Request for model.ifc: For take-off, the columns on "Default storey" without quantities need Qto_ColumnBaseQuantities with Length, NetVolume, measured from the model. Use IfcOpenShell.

First a look at what the model holds.

```python
import ifcopenshell
import ifcopenshell.util.element
import ifcopenshell.util.unit

model = ifcopenshell.open("model.ifc")
print(model.schema)
for unit_type in ("LENGTHUNIT", "AREAUNIT", "VOLUMEUNIT"):
    print(unit_type, ifcopenshell.util.unit.calculate_unit_scale(model, unit_type))
storey = next(s for s in model.by_type("IfcBuildingStorey") if s.Name == "Default storey")
columns = [e for e in ifcopenshell.util.element.get_decomposition(storey) if e.is_a("IfcColumn")]
for e in sorted(columns, key=lambda e: e.id()):
    print(e.id(), e.is_a(), e.Name, list(ifcopenshell.util.element.get_psets(e, qtos_only=True)), sep=" | ")
```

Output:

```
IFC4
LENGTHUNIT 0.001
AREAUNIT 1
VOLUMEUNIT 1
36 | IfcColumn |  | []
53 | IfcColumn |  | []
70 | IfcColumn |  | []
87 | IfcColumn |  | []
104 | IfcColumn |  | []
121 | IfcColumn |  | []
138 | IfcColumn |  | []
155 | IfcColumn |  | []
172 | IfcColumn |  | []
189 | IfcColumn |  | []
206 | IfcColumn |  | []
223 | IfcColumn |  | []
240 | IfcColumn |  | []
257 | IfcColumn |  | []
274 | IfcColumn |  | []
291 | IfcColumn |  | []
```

```python
import ifcopenshell
import ifcopenshell.api.pset
import ifcopenshell.geom
import ifcopenshell.util.element
import ifcopenshell.util.shape
import ifcopenshell.util.unit

model = ifcopenshell.open("model.ifc")
unit_scale = ifcopenshell.util.unit.calculate_unit_scale(model)
volume_scale = ifcopenshell.util.unit.calculate_unit_scale(model, "VOLUMEUNIT")
settings = ifcopenshell.geom.settings()

storey = next(s for s in model.by_type("IfcBuildingStorey") if s.Name == "Default storey")
columns = [e for e in ifcopenshell.util.element.get_decomposition(storey) if e.is_a("IfcColumn")]

for e in sorted(columns, key=lambda e: e.id()):
    if ifcopenshell.util.element.get_psets(e, qtos_only=True, should_inherit=False):
        continue
    # Geometry comes back in metres, in the element's own axes.
    shape = ifcopenshell.geom.create_shape(settings, e)
    values = {
        "Length": ifcopenshell.util.shape.get_z(shape.geometry) / unit_scale,
        "NetVolume": ifcopenshell.util.shape.get_volume(shape.geometry) / volume_scale,
    }
    qto = ifcopenshell.api.pset.add_qto(model, product=e, name="Qto_ColumnBaseQuantities")
    ifcopenshell.api.pset.edit_qto(model, qto=qto, properties=values)
    print(e.id(), {k: round(v, 3) for k, v in values.items()})

model.write("model-out.ifc")
```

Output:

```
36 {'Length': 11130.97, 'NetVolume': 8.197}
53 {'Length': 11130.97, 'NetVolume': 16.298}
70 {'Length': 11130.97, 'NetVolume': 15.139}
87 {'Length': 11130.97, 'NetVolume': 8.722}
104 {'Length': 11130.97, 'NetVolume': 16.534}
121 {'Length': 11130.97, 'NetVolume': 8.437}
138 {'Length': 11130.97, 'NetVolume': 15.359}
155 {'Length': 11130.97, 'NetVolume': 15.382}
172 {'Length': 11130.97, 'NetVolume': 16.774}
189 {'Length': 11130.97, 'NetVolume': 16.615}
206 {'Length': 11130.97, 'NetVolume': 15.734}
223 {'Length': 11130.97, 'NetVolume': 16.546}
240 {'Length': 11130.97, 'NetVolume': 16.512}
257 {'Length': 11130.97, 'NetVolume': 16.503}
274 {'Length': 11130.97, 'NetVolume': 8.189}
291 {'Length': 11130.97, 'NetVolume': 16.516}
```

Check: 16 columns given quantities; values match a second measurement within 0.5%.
